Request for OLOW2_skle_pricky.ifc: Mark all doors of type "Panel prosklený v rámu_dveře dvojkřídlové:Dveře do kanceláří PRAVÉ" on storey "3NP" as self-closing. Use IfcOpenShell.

First a look at what the model holds.

```python
import ifcopenshell
import ifcopenshell.util.element

model = ifcopenshell.open("OLOW2_skle_pricky.ifc")
print(model.schema)
storey = next(s for s in model.by_type("IfcBuildingStorey") if s.Name == "3NP")
doors = [e for e in ifcopenshell.util.element.get_decomposition(storey) if e.is_a("IfcDoor")]
seen = {}
for e in doors:
    element_type = ifcopenshell.util.element.get_type(e)
    key = (element_type.Name if element_type != e and element_type else None, ifcopenshell.util.element.get_pset(e, "Pset_DoorCommon", "SelfClosing"))
    seen[key] = seen.get(key, 0) + 1
for (name, value), count in sorted(seen.items(), key=str):
    print(count, "x", name, "|", value)
```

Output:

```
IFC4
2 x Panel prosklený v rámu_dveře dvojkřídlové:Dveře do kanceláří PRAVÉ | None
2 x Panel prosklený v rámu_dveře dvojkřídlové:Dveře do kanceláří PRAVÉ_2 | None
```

```python
import ifcopenshell
import ifcopenshell.api.pset
import ifcopenshell.util.element

model = ifcopenshell.open("OLOW2_skle_pricky.ifc")

storey = next(s for s in model.by_type("IfcBuildingStorey") if s.Name == "3NP")
doors = [e for e in ifcopenshell.util.element.get_decomposition(storey) if e.is_a("IfcDoor")]

count = 0
for e in doors:
    element_type = ifcopenshell.util.element.get_type(e)
    if element_type in (None, e) or element_type.Name != "Panel prosklený v rámu_dveře dvojkřídlové:Dveře do kanceláří PRAVÉ":
        continue
    # add_pset returns the element's existing set when there is one.
    pset = ifcopenshell.api.pset.add_pset(model, product=e, name="Pset_DoorCommon")
    ifcopenshell.api.pset.edit_pset(model, pset=pset, properties={"SelfClosing": True})
    count += 1

print(count, "doors updated")

model.write("OLOW2_skle_pricky_v2.ifc")
```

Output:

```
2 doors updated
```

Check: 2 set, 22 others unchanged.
